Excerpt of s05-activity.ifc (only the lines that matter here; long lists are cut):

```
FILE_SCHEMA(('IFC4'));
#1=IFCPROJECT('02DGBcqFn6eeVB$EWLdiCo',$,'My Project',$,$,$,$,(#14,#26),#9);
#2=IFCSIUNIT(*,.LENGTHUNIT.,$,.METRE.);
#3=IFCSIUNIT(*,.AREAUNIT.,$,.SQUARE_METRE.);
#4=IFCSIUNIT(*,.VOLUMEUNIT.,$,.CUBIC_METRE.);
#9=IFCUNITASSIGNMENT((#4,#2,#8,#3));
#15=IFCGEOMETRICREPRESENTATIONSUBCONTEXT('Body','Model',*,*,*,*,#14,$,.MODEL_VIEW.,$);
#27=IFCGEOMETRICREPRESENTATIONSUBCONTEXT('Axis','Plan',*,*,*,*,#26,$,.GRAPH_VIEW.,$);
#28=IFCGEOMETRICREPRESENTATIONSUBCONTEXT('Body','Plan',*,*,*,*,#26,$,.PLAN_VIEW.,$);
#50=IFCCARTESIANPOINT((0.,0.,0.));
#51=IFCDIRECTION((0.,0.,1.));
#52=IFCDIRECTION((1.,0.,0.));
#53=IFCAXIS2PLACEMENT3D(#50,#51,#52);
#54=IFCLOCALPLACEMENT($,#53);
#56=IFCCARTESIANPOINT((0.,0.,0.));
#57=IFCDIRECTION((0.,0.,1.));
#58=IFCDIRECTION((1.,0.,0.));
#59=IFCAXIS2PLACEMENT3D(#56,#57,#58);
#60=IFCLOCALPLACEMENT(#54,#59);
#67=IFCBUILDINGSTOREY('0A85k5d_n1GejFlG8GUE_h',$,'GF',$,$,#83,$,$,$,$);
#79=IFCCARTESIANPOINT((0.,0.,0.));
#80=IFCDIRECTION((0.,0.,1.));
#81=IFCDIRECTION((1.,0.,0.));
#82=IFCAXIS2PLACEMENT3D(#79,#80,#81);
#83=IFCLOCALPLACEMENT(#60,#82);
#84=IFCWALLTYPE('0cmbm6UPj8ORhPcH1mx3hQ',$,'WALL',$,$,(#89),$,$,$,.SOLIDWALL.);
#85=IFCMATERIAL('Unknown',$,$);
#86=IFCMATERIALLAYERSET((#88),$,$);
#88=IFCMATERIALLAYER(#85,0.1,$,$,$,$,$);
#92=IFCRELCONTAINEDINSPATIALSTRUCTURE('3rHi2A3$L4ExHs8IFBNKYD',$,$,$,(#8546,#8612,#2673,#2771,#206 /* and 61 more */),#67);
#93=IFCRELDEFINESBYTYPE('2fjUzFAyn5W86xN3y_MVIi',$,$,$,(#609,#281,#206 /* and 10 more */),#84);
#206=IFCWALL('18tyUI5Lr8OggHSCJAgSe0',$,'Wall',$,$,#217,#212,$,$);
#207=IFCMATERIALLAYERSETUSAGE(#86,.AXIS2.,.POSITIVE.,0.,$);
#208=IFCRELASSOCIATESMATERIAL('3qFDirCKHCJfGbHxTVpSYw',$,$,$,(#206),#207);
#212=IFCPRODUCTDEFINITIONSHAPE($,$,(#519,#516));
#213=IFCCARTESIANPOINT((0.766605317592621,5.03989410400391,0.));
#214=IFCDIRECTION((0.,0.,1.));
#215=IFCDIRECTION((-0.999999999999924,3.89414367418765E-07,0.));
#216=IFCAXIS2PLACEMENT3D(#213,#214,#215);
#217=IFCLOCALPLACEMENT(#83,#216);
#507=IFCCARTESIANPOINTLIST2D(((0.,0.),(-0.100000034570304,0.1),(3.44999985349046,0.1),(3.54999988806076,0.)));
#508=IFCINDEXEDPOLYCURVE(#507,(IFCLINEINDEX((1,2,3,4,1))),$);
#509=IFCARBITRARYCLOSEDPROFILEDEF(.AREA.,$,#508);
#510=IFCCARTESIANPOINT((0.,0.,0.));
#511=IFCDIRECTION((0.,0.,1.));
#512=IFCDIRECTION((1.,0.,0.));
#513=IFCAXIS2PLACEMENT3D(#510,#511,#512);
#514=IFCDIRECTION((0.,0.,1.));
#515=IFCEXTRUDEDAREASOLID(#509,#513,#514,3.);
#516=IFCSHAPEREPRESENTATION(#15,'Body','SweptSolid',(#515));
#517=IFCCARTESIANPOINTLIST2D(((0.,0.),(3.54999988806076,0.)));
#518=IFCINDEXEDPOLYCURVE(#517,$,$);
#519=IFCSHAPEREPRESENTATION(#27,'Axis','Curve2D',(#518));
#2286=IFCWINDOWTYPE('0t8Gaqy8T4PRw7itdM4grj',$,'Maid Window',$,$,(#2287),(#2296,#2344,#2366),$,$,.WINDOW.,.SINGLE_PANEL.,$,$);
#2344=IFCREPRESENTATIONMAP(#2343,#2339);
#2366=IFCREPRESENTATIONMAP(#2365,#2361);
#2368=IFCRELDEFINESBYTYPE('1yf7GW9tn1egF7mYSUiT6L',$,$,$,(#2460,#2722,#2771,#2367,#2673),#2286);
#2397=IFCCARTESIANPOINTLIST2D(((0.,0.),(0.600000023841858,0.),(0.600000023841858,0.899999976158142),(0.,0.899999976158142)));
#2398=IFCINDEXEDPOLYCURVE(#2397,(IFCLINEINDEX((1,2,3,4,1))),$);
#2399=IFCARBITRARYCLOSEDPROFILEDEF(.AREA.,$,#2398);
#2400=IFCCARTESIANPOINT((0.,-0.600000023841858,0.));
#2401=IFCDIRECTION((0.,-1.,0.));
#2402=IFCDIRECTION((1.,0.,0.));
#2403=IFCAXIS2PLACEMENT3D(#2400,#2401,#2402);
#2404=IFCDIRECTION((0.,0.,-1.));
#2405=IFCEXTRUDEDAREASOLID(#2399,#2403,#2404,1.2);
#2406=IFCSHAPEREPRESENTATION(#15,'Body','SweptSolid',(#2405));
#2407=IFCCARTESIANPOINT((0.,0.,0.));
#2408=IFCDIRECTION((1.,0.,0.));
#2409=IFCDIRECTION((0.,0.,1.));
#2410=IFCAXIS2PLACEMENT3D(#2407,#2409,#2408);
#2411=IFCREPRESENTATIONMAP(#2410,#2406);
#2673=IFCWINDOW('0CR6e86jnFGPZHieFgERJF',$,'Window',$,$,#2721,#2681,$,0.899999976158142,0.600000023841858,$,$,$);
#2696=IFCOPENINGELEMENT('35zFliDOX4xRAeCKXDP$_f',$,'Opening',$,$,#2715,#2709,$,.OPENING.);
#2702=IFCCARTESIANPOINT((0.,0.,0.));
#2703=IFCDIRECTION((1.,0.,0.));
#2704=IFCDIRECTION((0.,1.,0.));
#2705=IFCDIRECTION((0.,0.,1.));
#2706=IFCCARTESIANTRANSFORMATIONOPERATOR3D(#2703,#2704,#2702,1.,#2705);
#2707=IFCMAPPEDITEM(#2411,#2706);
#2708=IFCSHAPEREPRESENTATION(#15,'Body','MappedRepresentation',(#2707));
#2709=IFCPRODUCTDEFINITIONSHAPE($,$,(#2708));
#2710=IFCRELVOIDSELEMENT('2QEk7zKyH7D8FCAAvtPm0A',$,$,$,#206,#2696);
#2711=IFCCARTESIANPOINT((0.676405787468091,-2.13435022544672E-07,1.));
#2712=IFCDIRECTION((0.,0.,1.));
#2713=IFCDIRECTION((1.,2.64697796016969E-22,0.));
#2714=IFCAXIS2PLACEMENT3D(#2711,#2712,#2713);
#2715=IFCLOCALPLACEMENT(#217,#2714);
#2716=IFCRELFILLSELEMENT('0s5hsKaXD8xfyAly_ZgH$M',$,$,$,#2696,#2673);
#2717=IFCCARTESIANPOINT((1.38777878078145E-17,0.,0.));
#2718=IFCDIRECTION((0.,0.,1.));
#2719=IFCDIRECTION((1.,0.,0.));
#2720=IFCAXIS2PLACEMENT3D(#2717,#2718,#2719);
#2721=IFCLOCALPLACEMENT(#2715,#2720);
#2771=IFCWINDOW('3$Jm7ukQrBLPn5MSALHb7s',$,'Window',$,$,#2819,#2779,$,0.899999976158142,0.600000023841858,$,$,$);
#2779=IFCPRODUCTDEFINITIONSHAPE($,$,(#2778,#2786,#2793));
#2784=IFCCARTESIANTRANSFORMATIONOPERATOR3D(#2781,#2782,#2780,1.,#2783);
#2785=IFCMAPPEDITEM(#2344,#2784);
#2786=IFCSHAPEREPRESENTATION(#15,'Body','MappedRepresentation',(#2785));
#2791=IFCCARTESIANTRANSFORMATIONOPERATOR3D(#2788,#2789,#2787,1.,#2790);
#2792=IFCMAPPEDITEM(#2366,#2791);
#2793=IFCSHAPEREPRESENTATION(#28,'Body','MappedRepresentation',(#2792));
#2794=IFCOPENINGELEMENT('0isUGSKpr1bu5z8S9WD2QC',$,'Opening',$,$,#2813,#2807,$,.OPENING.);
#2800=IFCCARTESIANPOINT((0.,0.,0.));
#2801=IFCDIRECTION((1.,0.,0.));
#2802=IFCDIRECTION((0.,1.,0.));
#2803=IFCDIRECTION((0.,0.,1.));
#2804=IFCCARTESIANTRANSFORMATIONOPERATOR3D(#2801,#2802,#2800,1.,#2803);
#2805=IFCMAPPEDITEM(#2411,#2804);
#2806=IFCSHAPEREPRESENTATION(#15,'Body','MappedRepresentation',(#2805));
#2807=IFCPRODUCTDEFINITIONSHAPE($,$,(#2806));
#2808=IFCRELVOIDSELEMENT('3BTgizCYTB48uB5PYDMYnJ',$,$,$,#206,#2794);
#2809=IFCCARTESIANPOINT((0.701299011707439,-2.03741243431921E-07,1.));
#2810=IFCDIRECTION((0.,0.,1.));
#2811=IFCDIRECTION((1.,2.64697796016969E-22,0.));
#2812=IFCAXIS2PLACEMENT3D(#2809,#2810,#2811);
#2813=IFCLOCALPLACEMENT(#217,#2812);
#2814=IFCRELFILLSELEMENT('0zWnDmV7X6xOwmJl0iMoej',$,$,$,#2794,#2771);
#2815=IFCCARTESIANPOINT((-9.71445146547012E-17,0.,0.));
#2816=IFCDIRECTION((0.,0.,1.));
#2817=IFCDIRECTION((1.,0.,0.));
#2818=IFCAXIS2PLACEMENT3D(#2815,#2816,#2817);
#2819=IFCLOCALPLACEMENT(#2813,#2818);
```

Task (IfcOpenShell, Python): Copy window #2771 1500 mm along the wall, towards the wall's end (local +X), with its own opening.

```python
import ifcopenshell
import ifcopenshell.api.feature
import ifcopenshell.api.geometry
import ifcopenshell.api.root
import ifcopenshell.geom
import ifcopenshell.util.element
import ifcopenshell.util.placement
import ifcopenshell.util.shape
import ifcopenshell.util.unit

model = ifcopenshell.open("s05-activity.ifc")
unit_scale = ifcopenshell.util.unit.calculate_unit_scale(model)
settings = ifcopenshell.geom.settings()


def volume(element):
    """Net volume in cubic metres, openings subtracted."""
    shape = ifcopenshell.geom.create_shape(settings, element)
    return ifcopenshell.util.shape.get_volume(shape.geometry)


window = model.by_id(2771)
opening = window.FillsVoids[0].RelatingOpeningElement
wall = opening.VoidsElements[0].RelatingBuildingElement
before = volume(wall)
shift = ifcopenshell.util.placement.get_local_placement(wall.ObjectPlacement)[:3, 0] * 1.5 / unit_scale

# copy_class copies the void relationship, type, container and properties, but no geometry.
new_opening = ifcopenshell.api.root.copy_class(model, product=opening)
new_opening.Representation = ifcopenshell.util.element.copy_deep(
    model, opening.Representation, exclude=["IfcGeometricRepresentationContext", "IfcRepresentationMap"]
)
new_window = ifcopenshell.api.root.copy_class(model, product=window)
new_window.Representation = ifcopenshell.util.element.copy_deep(
    model, window.Representation, exclude=["IfcGeometricRepresentationContext", "IfcRepresentationMap"]
)
ifcopenshell.api.feature.add_filling(model, opening=new_opening, element=new_window)

for old, new in ((opening, new_opening), (window, new_window)):
    matrix = ifcopenshell.util.placement.get_local_placement(old.ObjectPlacement)
    matrix[:3, 3] += shift
    ifcopenshell.api.geometry.edit_object_placement(model, product=new, matrix=matrix, is_si=False)

after = volume(wall)

print(f"wall volume {before:.3f} -> {after:.3f} m3")

model.write("s05-activity-out.ifc")
```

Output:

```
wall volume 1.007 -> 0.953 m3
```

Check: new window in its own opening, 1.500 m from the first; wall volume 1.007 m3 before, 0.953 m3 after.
